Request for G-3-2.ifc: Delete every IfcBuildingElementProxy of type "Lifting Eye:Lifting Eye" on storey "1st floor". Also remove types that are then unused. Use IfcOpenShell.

First a look at what the model holds.

```python
import ifcopenshell
import ifcopenshell.util.element

model = ifcopenshell.open("G-3-2.ifc")
print(model.schema)
storey = next(s for s in model.by_type("IfcBuildingStorey") if s.Name == "1st floor")
proxies = [e for e in ifcopenshell.util.element.get_decomposition(storey) if e.is_a("IfcBuildingElementProxy")]
seen = {}
for e in proxies:
    element_type = ifcopenshell.util.element.get_type(e)
    name = element_type.Name if element_type not in (None, e) else None
    seen[name] = seen.get(name, 0) + 1
for name, count in sorted(seen.items(), key=str):
    print(count, "x", name)
```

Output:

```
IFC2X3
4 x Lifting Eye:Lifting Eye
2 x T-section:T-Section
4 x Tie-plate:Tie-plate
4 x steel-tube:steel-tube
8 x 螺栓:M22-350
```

```python
import ifcopenshell
import ifcopenshell.api.root
import ifcopenshell.util.element

model = ifcopenshell.open("G-3-2.ifc")

storey = next(s for s in model.by_type("IfcBuildingStorey") if s.Name == "1st floor")
proxies = [e for e in ifcopenshell.util.element.get_decomposition(storey) if e.is_a("IfcBuildingElementProxy")]
targets = [e for e in proxies if (t := ifcopenshell.util.element.get_type(e)) not in (None, e) and t.Name == "Lifting Eye:Lifting Eye"]
types = {ifcopenshell.util.element.get_type(e) for e in targets} - {None, *targets}

for e in targets:
    ifcopenshell.api.root.remove_product(model, product=e)
print(len(targets), "removed")

unused = [t for t in types if not ifcopenshell.util.element.get_types(t)]
for t in unused:
    ifcopenshell.api.root.remove_product(model, product=t)
print(len(unused), "unused types removed")

model.write("G-3-2_v2.ifc")
```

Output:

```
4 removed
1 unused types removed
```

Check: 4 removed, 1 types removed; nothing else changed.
